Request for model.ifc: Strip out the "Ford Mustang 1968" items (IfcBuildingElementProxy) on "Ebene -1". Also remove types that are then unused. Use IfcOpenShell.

First a look at what the model holds.

```python
import ifcopenshell
import ifcopenshell.util.element

model = ifcopenshell.open("model.ifc")
print(model.schema)
storey = next(s for s in model.by_type("IfcBuildingStorey") if s.Name == "Ebene -1")
proxies = [e for e in ifcopenshell.util.element.get_decomposition(storey) if e.is_a("IfcBuildingElementProxy")]
seen = {}
for e in proxies:
    element_type = ifcopenshell.util.element.get_type(e)
    name = element_type.Name if element_type not in (None, e) else None
    seen[name] = seen.get(name, 0) + 1
for name, count in sorted(seen.items(), key=str):
    print(count, "x", name)
```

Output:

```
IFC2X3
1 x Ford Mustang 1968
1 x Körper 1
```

```python
import ifcopenshell
import ifcopenshell.api.root
import ifcopenshell.util.element

model = ifcopenshell.open("model.ifc")

storey = next(s for s in model.by_type("IfcBuildingStorey") if s.Name == "Ebene -1")
proxies = [e for e in ifcopenshell.util.element.get_decomposition(storey) if e.is_a("IfcBuildingElementProxy")]
targets = [e for e in proxies if (t := ifcopenshell.util.element.get_type(e)) not in (None, e) and t.Name == "Ford Mustang 1968"]
types = {ifcopenshell.util.element.get_type(e) for e in targets} - {None, *targets}

for e in targets:
    ifcopenshell.api.root.remove_product(model, product=e)
print(len(targets), "removed")

unused = [t for t in types if not ifcopenshell.util.element.get_types(t)]
for t in unused:
    ifcopenshell.api.root.remove_product(model, product=t)
print(len(unused), "unused types removed")

model.write("model_updated.ifc")
```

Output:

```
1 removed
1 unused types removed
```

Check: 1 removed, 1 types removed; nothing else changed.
